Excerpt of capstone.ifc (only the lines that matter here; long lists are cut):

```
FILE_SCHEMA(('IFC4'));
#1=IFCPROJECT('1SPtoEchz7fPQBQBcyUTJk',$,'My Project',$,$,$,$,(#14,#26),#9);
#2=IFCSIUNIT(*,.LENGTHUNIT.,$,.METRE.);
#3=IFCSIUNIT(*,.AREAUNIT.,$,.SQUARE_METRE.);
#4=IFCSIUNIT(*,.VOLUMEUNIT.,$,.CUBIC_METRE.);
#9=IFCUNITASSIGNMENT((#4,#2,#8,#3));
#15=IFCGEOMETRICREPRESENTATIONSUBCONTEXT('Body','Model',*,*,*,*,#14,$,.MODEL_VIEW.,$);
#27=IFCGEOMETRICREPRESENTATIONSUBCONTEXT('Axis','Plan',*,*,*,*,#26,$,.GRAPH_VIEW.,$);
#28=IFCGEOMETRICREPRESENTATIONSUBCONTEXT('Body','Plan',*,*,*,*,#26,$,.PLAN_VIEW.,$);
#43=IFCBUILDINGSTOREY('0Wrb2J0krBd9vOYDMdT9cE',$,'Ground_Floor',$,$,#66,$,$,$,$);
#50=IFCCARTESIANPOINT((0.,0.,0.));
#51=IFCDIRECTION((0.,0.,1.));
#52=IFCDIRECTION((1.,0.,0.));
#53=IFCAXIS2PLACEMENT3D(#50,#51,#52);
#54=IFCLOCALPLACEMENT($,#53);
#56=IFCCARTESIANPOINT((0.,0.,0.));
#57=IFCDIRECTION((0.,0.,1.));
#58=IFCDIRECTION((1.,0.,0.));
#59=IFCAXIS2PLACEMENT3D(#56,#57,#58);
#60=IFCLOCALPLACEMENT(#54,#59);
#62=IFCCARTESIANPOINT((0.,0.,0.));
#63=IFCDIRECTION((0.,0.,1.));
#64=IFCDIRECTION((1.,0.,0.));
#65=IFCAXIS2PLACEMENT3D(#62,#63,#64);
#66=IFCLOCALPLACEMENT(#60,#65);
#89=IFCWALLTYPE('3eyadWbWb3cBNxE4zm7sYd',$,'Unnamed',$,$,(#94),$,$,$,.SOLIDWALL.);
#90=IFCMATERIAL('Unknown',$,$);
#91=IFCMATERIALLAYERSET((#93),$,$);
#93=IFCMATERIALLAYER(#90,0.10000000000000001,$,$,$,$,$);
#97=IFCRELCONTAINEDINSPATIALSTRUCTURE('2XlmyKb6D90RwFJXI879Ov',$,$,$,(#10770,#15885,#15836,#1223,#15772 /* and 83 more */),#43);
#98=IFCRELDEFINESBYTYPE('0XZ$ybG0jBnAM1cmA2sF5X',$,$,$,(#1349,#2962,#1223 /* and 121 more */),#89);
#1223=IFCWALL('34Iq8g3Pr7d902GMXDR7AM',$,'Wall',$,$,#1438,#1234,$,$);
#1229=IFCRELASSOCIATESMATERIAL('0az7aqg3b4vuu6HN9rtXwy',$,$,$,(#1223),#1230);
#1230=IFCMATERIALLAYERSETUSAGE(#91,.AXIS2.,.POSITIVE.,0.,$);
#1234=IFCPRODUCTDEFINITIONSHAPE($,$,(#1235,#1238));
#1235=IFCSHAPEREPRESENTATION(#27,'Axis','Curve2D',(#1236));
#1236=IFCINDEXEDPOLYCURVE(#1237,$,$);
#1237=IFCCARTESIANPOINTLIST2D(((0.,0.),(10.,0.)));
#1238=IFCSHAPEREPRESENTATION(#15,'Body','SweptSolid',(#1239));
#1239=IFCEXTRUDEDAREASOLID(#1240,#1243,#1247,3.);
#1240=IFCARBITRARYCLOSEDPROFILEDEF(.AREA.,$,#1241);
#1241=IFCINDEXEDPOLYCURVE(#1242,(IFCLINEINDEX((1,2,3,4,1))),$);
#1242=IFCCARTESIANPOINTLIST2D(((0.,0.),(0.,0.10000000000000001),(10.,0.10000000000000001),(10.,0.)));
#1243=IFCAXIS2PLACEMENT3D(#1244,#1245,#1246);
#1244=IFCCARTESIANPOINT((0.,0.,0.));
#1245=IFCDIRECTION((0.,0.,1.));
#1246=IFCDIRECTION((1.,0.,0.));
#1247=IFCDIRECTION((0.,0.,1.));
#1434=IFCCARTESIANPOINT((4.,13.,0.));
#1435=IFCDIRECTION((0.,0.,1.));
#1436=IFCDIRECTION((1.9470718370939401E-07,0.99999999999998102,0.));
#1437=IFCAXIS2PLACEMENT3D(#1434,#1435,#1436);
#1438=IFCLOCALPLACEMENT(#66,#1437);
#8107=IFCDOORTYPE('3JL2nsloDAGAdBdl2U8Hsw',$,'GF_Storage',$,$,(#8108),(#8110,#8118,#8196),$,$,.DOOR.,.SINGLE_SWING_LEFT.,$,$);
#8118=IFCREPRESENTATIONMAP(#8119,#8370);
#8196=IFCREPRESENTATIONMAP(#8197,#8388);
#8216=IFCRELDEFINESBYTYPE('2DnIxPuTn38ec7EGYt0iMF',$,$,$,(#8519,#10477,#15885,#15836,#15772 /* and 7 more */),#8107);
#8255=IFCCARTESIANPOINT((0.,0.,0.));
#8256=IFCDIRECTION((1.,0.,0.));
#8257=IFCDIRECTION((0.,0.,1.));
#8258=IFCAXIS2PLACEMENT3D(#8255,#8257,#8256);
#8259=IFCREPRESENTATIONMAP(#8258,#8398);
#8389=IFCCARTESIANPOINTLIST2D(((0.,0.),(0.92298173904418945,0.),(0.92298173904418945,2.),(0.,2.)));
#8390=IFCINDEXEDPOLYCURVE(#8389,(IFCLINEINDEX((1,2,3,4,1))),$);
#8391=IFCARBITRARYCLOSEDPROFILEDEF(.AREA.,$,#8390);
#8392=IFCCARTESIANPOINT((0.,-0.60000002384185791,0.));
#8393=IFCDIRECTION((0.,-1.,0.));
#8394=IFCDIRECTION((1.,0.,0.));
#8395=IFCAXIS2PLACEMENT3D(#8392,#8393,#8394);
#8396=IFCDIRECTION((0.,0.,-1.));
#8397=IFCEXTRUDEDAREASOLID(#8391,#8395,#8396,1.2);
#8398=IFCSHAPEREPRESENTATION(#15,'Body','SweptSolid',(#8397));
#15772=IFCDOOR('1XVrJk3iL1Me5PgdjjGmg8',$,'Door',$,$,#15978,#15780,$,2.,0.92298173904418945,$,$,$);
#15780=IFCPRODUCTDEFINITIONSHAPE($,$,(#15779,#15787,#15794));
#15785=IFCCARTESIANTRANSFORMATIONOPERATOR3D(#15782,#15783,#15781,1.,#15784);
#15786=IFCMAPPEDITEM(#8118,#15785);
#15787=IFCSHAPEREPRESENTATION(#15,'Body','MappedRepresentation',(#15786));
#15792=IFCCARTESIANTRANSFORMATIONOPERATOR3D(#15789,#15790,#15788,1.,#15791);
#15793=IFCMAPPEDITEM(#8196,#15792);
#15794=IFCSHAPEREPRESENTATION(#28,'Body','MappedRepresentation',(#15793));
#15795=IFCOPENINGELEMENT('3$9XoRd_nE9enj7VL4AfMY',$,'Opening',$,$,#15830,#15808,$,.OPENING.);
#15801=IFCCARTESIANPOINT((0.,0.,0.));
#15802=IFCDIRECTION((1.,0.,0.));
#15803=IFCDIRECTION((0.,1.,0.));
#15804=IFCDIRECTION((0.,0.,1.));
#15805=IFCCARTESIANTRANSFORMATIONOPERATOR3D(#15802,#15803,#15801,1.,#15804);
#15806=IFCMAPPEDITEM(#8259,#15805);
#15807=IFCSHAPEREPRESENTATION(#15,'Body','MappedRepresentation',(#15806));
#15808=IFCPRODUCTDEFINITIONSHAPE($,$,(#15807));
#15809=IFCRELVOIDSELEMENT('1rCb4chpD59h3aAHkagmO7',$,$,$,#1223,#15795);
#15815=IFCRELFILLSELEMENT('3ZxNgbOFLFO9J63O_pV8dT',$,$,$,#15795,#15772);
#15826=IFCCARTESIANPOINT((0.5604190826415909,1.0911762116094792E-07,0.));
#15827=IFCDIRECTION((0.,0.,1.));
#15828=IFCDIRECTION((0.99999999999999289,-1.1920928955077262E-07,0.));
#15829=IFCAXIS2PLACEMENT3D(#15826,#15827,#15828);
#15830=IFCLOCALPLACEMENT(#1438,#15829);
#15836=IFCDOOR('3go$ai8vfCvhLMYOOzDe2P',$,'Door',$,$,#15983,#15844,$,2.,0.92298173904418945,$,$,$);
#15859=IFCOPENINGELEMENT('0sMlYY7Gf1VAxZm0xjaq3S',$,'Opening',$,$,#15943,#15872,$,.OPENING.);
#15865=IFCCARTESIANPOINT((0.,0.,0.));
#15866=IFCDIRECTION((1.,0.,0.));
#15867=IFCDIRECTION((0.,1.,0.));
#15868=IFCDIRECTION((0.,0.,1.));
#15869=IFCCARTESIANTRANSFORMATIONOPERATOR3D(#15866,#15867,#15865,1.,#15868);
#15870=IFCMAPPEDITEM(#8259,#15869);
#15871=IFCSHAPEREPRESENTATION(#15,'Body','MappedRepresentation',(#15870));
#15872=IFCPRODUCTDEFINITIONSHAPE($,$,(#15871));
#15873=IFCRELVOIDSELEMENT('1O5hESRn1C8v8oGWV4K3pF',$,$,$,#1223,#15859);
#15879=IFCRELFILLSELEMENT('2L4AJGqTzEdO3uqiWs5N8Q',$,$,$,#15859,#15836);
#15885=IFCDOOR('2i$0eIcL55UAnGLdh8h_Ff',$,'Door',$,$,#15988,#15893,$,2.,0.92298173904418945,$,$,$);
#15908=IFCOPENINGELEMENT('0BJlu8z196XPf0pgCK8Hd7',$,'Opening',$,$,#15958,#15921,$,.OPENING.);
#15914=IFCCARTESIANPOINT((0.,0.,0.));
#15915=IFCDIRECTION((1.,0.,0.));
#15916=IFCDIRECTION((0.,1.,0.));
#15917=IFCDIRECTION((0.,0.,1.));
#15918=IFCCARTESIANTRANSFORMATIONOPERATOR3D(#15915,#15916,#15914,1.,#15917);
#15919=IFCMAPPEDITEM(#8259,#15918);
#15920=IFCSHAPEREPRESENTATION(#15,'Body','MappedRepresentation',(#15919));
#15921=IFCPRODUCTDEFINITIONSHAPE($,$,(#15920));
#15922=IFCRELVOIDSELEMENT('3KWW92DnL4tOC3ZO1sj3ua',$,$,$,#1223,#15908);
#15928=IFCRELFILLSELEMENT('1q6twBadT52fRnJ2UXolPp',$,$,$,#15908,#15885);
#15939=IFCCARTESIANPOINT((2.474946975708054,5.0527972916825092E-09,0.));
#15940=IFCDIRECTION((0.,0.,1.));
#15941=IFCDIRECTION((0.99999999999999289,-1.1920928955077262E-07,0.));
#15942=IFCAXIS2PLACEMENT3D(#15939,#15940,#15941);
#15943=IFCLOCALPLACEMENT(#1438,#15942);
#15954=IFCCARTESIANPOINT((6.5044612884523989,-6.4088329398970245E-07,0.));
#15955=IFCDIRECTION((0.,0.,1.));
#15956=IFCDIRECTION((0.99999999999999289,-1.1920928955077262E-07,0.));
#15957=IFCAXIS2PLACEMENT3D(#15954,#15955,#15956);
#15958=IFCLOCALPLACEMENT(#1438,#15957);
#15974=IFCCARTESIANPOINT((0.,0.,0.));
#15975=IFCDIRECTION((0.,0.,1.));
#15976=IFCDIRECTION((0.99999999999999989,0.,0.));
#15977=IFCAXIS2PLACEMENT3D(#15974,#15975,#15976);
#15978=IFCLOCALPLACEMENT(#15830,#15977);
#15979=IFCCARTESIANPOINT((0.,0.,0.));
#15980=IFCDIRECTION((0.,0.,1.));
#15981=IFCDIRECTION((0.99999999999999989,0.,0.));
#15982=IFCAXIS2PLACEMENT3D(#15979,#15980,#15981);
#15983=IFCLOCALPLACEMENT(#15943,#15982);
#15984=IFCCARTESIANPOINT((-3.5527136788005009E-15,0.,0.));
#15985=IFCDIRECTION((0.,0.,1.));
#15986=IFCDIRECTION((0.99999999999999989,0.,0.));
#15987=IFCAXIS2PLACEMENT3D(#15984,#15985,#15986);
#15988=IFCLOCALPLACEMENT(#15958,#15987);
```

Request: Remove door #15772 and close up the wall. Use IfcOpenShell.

```python
import ifcopenshell
import ifcopenshell.api.feature
import ifcopenshell.api.root
import ifcopenshell.geom
import ifcopenshell.util.shape

model = ifcopenshell.open("capstone.ifc")
settings = ifcopenshell.geom.settings()


def volume(element):
    """Net volume in cubic metres, openings subtracted."""
    shape = ifcopenshell.geom.create_shape(settings, element)
    return ifcopenshell.util.shape.get_volume(shape.geometry)


door = model.by_guid("1XVrJk3iL1Me5PgdjjGmg8")
opening = door.FillsVoids[0].RelatingOpeningElement
wall = opening.VoidsElements[0].RelatingBuildingElement
before = volume(wall)

ifcopenshell.api.root.remove_product(model, product=door)
ifcopenshell.api.feature.remove_feature(model, feature=opening)

after = volume(wall)

print(f"wall volume {before:.3f} -> {after:.3f} m3")

model.write("capstone_rev.ifc")
```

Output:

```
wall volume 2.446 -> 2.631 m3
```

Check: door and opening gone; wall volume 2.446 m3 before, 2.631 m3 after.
